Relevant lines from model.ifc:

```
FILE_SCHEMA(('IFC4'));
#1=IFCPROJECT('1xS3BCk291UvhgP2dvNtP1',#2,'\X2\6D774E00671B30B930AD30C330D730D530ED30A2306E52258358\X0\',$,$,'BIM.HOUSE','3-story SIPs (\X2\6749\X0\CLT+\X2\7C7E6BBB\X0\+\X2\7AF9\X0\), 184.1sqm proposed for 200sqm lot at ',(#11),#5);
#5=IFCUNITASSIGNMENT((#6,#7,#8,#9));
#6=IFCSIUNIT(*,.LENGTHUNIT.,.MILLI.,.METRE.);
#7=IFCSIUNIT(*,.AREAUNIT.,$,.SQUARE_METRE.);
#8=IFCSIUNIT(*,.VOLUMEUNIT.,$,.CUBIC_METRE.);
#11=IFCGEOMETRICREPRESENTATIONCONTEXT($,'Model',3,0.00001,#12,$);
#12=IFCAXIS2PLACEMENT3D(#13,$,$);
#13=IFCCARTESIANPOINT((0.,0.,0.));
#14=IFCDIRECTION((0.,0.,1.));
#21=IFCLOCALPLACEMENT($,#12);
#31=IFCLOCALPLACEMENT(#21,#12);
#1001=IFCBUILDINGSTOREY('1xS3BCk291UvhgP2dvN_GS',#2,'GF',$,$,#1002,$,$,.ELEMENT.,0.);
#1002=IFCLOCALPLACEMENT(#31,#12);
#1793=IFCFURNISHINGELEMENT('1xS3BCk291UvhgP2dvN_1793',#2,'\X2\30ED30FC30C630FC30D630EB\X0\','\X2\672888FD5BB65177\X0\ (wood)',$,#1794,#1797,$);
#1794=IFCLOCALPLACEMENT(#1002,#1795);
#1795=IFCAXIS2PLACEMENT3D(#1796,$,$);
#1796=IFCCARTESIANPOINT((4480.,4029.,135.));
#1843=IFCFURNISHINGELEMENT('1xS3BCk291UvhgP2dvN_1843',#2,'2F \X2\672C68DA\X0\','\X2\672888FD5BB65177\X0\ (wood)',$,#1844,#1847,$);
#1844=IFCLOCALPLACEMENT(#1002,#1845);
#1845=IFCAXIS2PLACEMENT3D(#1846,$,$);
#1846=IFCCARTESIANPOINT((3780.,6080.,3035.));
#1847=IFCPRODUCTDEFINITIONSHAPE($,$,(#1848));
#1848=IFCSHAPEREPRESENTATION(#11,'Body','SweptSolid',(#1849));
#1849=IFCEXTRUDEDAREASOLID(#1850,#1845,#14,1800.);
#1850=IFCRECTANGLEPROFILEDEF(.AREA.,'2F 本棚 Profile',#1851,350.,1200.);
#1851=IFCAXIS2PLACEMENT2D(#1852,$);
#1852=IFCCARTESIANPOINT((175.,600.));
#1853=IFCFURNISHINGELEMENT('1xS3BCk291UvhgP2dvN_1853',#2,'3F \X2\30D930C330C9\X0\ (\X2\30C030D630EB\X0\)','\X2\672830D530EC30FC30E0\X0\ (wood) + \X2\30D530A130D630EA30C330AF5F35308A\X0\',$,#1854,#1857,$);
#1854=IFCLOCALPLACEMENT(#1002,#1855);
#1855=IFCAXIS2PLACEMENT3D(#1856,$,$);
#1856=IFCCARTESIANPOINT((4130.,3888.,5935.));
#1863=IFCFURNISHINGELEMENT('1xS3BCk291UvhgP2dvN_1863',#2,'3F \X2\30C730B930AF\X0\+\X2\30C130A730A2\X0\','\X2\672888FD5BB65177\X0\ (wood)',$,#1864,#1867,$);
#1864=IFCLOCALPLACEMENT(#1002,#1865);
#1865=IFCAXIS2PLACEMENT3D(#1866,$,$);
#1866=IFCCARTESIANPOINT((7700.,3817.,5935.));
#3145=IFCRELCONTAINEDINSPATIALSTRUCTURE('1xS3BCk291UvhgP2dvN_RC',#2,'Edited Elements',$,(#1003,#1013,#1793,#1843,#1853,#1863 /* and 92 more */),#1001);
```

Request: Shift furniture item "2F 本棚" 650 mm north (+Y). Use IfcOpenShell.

```python
import ifcopenshell
import ifcopenshell.api.geometry
import ifcopenshell.util.placement
import ifcopenshell.util.unit

model = ifcopenshell.open("model.ifc")
unit_scale = ifcopenshell.util.unit.calculate_unit_scale(model)

item = model.by_id(1843)
matrix = ifcopenshell.util.placement.get_local_placement(item.ObjectPlacement)
matrix[1, 3] += 0.65 / unit_scale
ifcopenshell.api.geometry.edit_object_placement(model, product=item, matrix=matrix, is_si=False)

print(ifcopenshell.util.placement.get_local_placement(item.ObjectPlacement).round(3) + 0.0)

model.write("model-out.ifc")
```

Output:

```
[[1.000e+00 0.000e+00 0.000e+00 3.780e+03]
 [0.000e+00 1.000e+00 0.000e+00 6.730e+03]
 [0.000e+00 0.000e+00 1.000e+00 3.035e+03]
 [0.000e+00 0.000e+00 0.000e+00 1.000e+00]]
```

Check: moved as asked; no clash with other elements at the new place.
